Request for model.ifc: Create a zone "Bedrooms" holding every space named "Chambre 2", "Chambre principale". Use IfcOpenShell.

First a look at what the model holds.

```python
import ifcopenshell

model = ifcopenshell.open("model.ifc")
print(model.schema)
seen = {}
for space in model.by_type("IfcSpace"):
    seen[space.LongName] = seen.get(space.LongName, 0) + 1
for name, count in sorted(seen.items(), key=str):
    print(count, "x", name)
print("zones:", [z.Name for z in model.by_type("IfcZone")][:20])
```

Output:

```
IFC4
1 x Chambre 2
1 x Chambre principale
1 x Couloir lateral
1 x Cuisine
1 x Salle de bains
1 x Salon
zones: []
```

```python
import ifcopenshell
import ifcopenshell.api.group
import ifcopenshell.api.root

model = ifcopenshell.open("model.ifc")

names = {"Chambre 2", "Chambre principale"}
spaces = [s for s in model.by_type("IfcSpace") if s.LongName in names]

zone = ifcopenshell.api.root.create_entity(model, ifc_class="IfcZone", name="Bedrooms")
ifcopenshell.api.group.assign_group(model, products=spaces, group=zone)
print(len(spaces), "spaces in", zone.Name)

model.write("model_rev.ifc")
```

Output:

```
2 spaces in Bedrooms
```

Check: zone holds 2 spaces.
